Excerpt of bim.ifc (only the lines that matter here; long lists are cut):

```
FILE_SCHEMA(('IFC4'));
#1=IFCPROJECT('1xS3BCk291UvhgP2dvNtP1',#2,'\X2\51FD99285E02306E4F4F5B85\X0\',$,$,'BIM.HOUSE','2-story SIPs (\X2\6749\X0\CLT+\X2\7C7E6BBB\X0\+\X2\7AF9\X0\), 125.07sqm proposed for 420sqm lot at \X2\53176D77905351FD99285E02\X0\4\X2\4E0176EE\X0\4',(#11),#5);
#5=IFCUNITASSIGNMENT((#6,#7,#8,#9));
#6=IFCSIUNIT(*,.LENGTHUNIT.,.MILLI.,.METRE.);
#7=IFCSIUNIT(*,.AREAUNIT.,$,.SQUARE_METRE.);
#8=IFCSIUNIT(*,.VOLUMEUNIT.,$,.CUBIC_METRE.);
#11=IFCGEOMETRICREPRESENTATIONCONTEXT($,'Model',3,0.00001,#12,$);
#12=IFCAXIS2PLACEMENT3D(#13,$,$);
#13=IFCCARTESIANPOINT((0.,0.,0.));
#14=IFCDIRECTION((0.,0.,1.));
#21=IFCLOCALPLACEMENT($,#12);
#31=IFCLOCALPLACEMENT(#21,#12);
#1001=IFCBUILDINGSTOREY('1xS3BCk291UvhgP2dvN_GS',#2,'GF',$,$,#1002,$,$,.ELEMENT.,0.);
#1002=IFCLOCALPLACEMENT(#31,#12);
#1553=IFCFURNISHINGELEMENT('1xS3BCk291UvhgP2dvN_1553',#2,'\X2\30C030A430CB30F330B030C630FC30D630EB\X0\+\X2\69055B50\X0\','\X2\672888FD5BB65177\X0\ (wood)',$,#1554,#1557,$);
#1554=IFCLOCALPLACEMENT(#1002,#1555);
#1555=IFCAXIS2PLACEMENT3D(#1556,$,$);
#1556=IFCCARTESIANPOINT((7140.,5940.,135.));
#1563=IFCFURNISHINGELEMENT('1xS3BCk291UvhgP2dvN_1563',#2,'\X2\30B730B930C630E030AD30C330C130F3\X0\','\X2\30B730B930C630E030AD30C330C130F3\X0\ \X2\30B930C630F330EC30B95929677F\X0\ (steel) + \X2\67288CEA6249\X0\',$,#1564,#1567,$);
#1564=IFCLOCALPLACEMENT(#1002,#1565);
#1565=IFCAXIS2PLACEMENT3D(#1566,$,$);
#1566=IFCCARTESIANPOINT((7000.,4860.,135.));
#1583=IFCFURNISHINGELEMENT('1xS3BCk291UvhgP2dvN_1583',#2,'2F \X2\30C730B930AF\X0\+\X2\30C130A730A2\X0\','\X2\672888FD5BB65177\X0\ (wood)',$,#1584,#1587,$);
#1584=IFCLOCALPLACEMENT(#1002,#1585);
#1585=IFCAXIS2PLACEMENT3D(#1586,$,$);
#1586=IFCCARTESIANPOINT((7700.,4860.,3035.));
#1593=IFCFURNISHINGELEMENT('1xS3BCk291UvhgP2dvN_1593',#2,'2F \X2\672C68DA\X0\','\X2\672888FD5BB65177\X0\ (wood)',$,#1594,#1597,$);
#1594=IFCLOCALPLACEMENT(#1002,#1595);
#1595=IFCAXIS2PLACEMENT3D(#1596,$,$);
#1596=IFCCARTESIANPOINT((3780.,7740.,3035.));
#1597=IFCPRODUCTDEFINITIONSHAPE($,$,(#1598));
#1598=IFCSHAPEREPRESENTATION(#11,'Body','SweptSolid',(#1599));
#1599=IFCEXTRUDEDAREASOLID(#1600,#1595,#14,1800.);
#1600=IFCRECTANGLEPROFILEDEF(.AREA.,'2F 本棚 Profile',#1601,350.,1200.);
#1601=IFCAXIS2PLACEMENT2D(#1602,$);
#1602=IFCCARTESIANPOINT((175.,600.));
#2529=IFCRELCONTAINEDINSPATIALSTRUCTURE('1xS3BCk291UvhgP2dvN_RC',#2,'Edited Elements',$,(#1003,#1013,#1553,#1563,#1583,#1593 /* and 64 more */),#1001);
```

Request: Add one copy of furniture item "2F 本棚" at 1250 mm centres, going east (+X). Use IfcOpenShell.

```python
import numpy as np
import ifcopenshell
import ifcopenshell.api.geometry
import ifcopenshell.api.root
import ifcopenshell.util.element
import ifcopenshell.util.placement
import ifcopenshell.util.unit

model = ifcopenshell.open("bim.ifc")
unit_scale = ifcopenshell.util.unit.calculate_unit_scale(model)


def reuse_history(source, copy):
    """copy_class also copies each property set's owner history, people and application; keep the originals."""
    for rel in copy.IsDefinedBy:
        if rel.is_a("IfcRelDefinesByProperties") and (history := rel.RelatingPropertyDefinition.OwnerHistory):
            rel.RelatingPropertyDefinition.OwnerHistory = source.OwnerHistory
            ifcopenshell.util.element.remove_deep2(model, history)


source = model.by_id(1593)
base = ifcopenshell.util.placement.get_local_placement(source.ObjectPlacement)
step = np.array([1.0, 0.0, 0.0]) * 1.25 / unit_scale

for i in range(1, 2):
    copy = ifcopenshell.api.root.copy_class(model, product=source)
    copy.Representation = ifcopenshell.util.element.copy_deep(
        model, source.Representation, exclude=["IfcGeometricRepresentationContext", "IfcRepresentationMap"]
    )
    reuse_history(source, copy)
    matrix = base.copy()
    matrix[:3, 3] += i * step
    print("added at", matrix[:3, 3].round(3) + 0.0)
    ifcopenshell.api.geometry.edit_object_placement(model, product=copy, matrix=matrix, is_si=False)

model.write("bim-out.ifc")
```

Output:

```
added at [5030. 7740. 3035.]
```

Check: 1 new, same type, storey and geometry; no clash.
